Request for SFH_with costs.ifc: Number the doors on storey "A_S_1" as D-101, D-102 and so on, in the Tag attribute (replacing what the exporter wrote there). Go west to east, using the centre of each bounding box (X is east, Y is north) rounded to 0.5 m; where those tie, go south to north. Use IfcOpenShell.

First a look at what the model holds.

```python
import ifcopenshell
import ifcopenshell.util.element
import ifcopenshell.util.placement

model = ifcopenshell.open("SFH_with costs.ifc")
print(model.schema)
storey = next(s for s in model.by_type("IfcBuildingStorey") if s.Name == "A_S_1")
doors = [e for e in ifcopenshell.util.element.get_decomposition(storey) if e.is_a("IfcDoor")]
for e in sorted(doors, key=lambda e: e.id()):
    origin = ifcopenshell.util.placement.get_local_placement(e.ObjectPlacement)[:3, 3]
    print(e.id(), e.Tag, e.Name, origin.round(2) + 0.0, sep=" | ")
```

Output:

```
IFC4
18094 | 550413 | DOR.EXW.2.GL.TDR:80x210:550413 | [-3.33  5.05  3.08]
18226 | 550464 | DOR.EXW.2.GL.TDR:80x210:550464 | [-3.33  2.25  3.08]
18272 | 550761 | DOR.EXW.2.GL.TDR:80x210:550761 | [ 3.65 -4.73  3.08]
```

```python
import ifcopenshell
import ifcopenshell.geom
import ifcopenshell.util.element
import ifcopenshell.util.shape

model = ifcopenshell.open("SFH_with costs.ifc")
settings = ifcopenshell.geom.settings()
settings.set("use-world-coords", True)


def centre(element):
    shape = ifcopenshell.geom.create_shape(settings, element)
    return ifcopenshell.util.shape.get_bbox_centroid(shape.geometry)


storey = next(s for s in model.by_type("IfcBuildingStorey") if s.Name == "A_S_1")
doors = [e for e in ifcopenshell.util.element.get_decomposition(storey) if e.is_a("IfcDoor")]

# Insertion points can sit at a corner or the storey origin, so sort by the geometry (in metres).
centres = {e: centre(e) for e in doors}
doors.sort(key=lambda e: (round(centres[e][0] / 0.5), centres[e][1]))

for i, e in enumerate(doors, start=1):
    number = f"D-1{i:02d}"
    e.Tag = number
    print(e.id(), number)

model.write("SFH_with costs_v2.ifc")
```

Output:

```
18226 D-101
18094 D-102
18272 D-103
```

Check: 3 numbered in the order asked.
